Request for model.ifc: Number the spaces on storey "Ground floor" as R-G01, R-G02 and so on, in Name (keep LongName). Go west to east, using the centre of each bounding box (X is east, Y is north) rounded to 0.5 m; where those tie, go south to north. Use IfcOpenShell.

First a look at what the model holds.

```python
import ifcopenshell
import ifcopenshell.util.element
import ifcopenshell.util.placement

model = ifcopenshell.open("model.ifc")
print(model.schema)
storey = next(s for s in model.by_type("IfcBuildingStorey") if s.Name == "Ground floor")
spaces = [e for e in ifcopenshell.util.element.get_decomposition(storey) if e.is_a("IfcSpace")]
for e in sorted(spaces, key=lambda e: e.id()):
    origin = ifcopenshell.util.placement.get_local_placement(e.ObjectPlacement)[:3, 3]
    print(e.id(), e.Name, e.LongName, origin.round(2) + 0.0, sep=" | ")
```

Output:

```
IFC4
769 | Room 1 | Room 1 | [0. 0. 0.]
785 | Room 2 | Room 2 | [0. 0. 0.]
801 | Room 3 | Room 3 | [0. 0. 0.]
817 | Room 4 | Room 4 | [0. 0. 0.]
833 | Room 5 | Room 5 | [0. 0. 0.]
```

```python
import ifcopenshell
import ifcopenshell.geom
import ifcopenshell.util.element
import ifcopenshell.util.shape

model = ifcopenshell.open("model.ifc")
settings = ifcopenshell.geom.settings()
settings.set("use-world-coords", True)


def centre(element):
    shape = ifcopenshell.geom.create_shape(settings, element)
    return ifcopenshell.util.shape.get_bbox_centroid(shape.geometry)


storey = next(s for s in model.by_type("IfcBuildingStorey") if s.Name == "Ground floor")
spaces = [e for e in ifcopenshell.util.element.get_decomposition(storey) if e.is_a("IfcSpace")]

# Insertion points can sit at a corner or the storey origin, so sort by the geometry (in metres).
centres = {e: centre(e) for e in spaces}
spaces.sort(key=lambda e: (round(centres[e][0] / 0.5), centres[e][1]))

for i, e in enumerate(spaces, start=1):
    number = f"R-G{i:02d}"
    e.Name = number
    print(e.id(), number)

model.write("model_edited.ifc")
```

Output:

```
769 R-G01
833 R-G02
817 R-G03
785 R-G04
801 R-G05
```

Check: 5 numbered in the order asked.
